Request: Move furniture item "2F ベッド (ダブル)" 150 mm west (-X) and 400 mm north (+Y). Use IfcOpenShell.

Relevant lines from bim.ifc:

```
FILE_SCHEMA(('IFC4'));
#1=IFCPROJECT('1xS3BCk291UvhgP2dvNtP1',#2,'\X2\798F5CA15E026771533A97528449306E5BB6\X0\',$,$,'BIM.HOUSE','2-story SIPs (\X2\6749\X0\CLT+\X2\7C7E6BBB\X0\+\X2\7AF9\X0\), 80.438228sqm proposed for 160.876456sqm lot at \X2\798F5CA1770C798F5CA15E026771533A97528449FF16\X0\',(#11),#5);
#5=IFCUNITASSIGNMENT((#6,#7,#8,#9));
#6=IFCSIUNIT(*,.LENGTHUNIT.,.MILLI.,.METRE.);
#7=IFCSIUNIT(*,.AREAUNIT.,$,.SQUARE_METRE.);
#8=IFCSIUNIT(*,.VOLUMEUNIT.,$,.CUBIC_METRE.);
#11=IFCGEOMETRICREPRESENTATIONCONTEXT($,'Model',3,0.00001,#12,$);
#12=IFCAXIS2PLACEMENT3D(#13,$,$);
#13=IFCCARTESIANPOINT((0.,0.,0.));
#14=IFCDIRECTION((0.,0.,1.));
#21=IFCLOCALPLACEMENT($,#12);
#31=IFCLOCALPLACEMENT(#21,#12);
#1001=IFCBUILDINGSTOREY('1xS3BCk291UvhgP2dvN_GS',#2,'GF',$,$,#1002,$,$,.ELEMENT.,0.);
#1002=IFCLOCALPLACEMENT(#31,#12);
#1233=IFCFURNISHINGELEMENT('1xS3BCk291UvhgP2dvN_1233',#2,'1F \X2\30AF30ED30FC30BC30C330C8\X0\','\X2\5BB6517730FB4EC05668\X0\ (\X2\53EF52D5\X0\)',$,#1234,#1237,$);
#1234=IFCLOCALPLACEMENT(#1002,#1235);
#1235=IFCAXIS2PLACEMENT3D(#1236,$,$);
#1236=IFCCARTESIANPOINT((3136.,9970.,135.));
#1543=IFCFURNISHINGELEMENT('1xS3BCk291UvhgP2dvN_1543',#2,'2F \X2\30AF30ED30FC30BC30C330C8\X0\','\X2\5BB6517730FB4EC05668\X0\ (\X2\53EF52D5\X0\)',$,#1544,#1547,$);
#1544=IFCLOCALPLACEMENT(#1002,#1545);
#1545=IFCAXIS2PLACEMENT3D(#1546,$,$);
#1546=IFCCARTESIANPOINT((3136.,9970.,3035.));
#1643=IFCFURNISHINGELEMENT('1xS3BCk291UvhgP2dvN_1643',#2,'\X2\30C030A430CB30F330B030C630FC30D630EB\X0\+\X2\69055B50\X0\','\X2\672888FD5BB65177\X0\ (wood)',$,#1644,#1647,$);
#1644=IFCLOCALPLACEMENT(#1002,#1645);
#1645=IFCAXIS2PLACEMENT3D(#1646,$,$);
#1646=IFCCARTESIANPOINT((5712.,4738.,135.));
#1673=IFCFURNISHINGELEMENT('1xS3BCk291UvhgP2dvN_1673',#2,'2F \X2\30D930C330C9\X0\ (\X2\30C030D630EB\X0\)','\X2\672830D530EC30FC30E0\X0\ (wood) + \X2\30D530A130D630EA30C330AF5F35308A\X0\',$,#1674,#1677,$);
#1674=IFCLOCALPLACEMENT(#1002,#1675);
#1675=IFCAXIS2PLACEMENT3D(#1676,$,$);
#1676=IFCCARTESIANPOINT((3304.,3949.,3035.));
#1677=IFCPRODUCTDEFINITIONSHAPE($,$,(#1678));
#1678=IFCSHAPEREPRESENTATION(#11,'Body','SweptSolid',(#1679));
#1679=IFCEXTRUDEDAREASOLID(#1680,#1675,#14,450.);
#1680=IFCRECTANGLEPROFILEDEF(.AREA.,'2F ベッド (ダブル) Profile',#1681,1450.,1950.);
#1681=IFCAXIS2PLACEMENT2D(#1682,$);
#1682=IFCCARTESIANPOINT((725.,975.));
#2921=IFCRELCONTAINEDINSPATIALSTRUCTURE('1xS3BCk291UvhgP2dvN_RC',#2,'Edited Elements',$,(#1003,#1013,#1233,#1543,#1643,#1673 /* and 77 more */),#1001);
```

```python
import ifcopenshell
import ifcopenshell.api.geometry
import ifcopenshell.util.placement
import ifcopenshell.util.unit

model = ifcopenshell.open("bim.ifc")
unit_scale = ifcopenshell.util.unit.calculate_unit_scale(model)

item = model.by_id(1673)
matrix = ifcopenshell.util.placement.get_local_placement(item.ObjectPlacement)
matrix[0, 3] -= 0.15 / unit_scale
matrix[1, 3] += 0.4 / unit_scale
ifcopenshell.api.geometry.edit_object_placement(model, product=item, matrix=matrix, is_si=False)

print(ifcopenshell.util.placement.get_local_placement(item.ObjectPlacement).round(3) + 0.0)

model.write("bim_updated.ifc")
```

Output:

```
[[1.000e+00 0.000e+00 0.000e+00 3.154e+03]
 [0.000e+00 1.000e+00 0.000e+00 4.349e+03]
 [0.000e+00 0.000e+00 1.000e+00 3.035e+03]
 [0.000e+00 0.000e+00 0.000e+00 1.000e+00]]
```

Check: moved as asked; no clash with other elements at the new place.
